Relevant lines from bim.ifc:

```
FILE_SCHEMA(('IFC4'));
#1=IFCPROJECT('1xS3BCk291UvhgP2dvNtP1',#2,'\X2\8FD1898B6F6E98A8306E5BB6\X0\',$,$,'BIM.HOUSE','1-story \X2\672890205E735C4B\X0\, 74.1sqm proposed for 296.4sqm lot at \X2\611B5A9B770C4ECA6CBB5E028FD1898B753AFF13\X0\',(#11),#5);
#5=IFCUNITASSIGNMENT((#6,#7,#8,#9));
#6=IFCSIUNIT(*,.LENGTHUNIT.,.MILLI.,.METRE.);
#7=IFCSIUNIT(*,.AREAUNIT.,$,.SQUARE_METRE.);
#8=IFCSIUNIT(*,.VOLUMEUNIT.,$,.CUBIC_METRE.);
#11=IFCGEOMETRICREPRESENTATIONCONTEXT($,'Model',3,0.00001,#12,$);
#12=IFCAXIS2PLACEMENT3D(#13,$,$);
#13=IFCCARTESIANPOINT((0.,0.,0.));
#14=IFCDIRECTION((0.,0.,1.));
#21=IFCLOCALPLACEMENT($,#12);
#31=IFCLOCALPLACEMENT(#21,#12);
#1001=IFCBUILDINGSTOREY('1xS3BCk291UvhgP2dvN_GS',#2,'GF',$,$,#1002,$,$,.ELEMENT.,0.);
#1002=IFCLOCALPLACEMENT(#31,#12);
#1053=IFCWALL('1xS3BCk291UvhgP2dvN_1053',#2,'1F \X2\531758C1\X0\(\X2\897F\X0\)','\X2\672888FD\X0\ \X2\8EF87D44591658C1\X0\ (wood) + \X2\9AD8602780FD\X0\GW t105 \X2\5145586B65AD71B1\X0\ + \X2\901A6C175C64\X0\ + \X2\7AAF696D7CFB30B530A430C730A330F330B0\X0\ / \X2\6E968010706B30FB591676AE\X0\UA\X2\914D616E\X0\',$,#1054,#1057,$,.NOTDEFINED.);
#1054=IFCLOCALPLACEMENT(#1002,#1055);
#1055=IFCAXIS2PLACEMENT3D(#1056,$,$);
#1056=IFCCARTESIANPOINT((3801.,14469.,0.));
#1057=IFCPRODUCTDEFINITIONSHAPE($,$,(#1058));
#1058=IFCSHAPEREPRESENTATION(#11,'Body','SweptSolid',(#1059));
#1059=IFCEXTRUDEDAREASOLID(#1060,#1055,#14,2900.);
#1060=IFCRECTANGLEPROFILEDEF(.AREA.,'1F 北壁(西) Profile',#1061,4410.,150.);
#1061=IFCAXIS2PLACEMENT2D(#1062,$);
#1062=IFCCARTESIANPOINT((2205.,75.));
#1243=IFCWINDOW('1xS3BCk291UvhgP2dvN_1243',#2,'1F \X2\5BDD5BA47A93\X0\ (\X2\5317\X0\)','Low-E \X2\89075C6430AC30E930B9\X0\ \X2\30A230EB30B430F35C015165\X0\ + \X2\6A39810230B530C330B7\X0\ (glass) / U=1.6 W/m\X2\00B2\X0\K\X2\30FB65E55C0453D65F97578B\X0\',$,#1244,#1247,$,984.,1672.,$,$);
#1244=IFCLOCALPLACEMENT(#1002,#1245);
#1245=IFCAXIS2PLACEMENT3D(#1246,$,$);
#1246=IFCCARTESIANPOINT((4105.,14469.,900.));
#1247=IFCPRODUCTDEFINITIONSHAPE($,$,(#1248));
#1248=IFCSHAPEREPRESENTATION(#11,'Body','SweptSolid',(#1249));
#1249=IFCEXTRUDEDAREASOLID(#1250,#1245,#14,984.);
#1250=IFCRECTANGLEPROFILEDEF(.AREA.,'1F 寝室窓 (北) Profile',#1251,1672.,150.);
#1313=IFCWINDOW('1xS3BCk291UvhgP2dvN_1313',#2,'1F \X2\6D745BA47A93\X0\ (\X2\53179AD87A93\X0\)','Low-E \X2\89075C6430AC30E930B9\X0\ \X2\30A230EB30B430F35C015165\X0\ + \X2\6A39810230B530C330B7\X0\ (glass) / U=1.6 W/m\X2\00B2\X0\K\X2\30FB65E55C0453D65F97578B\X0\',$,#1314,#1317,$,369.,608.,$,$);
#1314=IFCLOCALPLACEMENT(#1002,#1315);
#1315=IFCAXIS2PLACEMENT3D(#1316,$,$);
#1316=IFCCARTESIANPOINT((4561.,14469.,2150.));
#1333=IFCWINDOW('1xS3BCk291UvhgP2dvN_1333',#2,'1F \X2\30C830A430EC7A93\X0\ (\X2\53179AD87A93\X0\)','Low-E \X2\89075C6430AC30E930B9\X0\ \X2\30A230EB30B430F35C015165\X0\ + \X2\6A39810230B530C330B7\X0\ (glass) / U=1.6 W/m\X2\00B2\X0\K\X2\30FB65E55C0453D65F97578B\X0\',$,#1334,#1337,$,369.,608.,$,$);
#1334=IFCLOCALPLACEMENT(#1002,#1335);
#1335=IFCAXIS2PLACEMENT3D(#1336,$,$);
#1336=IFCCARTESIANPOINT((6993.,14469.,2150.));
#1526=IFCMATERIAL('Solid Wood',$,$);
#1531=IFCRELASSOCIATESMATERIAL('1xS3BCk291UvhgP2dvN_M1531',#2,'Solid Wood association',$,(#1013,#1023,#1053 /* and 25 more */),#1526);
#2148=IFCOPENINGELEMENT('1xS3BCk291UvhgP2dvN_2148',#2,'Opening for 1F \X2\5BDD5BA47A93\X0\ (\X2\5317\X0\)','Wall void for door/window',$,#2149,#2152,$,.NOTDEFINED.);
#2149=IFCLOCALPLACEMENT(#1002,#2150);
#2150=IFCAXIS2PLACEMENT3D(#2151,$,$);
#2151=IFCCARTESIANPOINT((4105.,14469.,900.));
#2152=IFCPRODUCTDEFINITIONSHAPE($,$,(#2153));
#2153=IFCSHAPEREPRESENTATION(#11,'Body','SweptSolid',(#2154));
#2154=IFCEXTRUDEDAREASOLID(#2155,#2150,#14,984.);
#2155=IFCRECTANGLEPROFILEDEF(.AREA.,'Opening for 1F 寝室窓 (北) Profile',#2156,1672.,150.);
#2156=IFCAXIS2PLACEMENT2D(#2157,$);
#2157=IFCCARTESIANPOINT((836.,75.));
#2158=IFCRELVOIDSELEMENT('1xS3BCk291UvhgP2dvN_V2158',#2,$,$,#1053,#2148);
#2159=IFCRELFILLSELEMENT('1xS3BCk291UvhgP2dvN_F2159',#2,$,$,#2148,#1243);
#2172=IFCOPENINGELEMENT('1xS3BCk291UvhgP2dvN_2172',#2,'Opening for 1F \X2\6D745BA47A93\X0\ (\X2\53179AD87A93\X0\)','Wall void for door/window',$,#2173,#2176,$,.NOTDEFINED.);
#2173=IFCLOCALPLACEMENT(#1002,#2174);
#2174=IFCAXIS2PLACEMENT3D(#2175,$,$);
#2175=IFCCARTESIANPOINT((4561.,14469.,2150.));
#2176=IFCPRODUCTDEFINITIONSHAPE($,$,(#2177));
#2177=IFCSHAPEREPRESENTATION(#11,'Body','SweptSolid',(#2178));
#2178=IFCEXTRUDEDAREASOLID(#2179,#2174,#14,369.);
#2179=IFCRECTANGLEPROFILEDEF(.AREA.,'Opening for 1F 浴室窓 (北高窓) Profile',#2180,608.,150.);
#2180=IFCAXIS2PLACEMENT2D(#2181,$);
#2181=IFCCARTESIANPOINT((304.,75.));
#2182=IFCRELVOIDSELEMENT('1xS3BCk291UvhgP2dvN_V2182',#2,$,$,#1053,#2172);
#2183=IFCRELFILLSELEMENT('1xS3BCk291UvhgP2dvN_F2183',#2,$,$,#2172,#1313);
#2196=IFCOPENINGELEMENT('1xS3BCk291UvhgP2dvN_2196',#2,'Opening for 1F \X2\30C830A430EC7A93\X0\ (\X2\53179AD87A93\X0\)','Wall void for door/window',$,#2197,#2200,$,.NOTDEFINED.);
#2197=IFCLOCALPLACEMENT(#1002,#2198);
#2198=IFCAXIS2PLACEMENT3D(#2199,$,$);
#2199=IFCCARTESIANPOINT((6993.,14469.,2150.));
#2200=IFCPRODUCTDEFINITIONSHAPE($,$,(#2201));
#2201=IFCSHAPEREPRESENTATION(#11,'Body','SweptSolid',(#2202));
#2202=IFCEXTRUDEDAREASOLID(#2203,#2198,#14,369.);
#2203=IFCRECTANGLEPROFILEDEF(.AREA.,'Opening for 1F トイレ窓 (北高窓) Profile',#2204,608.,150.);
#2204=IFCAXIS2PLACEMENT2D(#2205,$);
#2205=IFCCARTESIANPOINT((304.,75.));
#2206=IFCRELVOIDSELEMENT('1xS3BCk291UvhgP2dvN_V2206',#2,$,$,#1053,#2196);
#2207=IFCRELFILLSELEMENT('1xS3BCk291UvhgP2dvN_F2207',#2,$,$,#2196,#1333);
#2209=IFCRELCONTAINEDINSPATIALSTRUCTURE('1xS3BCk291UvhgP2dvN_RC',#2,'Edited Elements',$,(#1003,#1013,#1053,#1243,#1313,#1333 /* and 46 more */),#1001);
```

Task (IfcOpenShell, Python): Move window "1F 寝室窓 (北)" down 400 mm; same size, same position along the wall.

```python
import numpy as np
import ifcopenshell
import ifcopenshell.api.geometry
import ifcopenshell.util.placement
import ifcopenshell.util.unit

model = ifcopenshell.open("bim.ifc")
unit_scale = ifcopenshell.util.unit.calculate_unit_scale(model)

window = model.by_guid("1xS3BCk291UvhgP2dvN_1243")
opening = window.FillsVoids[0].RelatingOpeningElement
dz = -0.4 / unit_scale

shift = np.array([0.0, 0.0, dz])
# The window is not placed relative to its opening, so move both.
for product in (opening, window):
    matrix = ifcopenshell.util.placement.get_local_placement(product.ObjectPlacement)
    matrix[:3, 3] += shift
    ifcopenshell.api.geometry.edit_object_placement(model, product=product, matrix=matrix, is_si=False)

print(f"moved by {dz * unit_scale:+.3f} m")

model.write("bim-out.ifc")
```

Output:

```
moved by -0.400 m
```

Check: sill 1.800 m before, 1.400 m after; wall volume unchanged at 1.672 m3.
